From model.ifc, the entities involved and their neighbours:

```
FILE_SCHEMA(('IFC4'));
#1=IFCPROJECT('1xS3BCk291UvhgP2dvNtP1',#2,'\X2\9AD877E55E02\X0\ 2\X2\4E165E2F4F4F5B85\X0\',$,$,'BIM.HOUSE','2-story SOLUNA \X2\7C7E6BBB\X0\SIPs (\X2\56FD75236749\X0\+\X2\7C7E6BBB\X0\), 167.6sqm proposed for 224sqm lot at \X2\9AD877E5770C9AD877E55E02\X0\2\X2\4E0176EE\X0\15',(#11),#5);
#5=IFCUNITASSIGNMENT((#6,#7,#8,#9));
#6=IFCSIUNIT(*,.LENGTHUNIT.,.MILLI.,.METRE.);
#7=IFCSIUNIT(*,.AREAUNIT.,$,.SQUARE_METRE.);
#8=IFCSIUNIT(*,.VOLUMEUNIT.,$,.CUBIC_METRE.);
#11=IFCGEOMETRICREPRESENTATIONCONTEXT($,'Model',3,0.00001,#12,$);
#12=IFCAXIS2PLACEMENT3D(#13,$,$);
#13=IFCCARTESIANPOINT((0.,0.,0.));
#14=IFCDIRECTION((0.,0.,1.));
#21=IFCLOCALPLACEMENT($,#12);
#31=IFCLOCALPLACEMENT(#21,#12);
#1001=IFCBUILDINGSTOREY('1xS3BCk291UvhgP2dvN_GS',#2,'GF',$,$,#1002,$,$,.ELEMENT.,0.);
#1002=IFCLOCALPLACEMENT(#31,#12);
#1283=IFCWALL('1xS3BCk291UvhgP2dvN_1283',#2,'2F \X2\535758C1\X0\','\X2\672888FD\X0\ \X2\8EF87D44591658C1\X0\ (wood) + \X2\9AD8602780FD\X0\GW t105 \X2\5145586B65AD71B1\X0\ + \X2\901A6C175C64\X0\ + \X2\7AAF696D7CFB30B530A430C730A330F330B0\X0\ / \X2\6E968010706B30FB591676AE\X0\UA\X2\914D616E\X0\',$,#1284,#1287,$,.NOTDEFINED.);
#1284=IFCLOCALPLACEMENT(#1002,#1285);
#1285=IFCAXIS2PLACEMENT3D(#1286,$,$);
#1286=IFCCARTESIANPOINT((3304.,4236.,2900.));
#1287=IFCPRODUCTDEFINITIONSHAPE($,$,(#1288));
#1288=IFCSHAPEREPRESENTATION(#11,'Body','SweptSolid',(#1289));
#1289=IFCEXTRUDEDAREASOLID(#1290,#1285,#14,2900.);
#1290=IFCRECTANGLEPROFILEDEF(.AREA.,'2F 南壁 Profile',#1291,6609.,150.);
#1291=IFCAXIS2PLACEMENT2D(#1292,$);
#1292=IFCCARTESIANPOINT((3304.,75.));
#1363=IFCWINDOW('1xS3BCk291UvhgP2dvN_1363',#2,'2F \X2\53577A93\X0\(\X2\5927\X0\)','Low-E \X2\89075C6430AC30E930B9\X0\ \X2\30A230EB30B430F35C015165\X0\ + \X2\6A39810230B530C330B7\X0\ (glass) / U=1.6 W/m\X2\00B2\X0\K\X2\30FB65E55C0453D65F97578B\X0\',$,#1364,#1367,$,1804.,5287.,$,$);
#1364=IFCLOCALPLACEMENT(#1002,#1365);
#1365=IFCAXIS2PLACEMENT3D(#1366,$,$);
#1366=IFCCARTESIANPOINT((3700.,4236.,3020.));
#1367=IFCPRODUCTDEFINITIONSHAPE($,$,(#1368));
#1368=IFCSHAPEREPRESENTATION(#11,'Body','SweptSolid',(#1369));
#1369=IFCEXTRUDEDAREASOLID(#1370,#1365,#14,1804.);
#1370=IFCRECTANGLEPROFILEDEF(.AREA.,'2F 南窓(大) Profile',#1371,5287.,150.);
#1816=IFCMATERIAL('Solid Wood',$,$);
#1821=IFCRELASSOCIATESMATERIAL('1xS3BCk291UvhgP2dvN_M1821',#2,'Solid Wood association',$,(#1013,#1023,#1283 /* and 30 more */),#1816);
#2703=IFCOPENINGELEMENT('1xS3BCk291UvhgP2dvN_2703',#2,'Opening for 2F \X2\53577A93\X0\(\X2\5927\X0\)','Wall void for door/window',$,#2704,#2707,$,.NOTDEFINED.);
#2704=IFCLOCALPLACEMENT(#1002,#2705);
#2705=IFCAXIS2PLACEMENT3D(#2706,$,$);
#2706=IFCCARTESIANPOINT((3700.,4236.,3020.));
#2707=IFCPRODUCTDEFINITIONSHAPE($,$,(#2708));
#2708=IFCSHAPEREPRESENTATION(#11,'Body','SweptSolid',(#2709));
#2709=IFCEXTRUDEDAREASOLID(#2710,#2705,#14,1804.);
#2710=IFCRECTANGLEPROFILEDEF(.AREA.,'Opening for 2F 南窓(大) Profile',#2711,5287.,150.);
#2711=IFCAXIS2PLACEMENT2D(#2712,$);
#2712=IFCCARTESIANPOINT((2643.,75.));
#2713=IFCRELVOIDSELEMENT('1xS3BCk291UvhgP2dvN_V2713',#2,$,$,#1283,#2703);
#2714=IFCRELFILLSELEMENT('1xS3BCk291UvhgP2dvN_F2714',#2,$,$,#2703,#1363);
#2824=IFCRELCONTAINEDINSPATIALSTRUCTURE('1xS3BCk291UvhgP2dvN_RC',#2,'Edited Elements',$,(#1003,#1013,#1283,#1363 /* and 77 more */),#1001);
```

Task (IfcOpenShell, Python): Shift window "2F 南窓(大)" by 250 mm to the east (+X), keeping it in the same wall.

```python
import ifcopenshell
import ifcopenshell.api.geometry
import ifcopenshell.util.placement
import ifcopenshell.util.unit

model = ifcopenshell.open("model.ifc")
unit_scale = ifcopenshell.util.unit.calculate_unit_scale(model)

window = model.by_id(1363)
opening = window.FillsVoids[0].RelatingOpeningElement
wall = opening.VoidsElements[0].RelatingBuildingElement

wall_matrix = ifcopenshell.util.placement.get_local_placement(wall.ObjectPlacement)
shift = wall_matrix[:3, 0] * 0.25 / unit_scale
before = ifcopenshell.util.placement.get_local_placement(window.ObjectPlacement)[:3, 3].copy()

# The window is not placed relative to its opening, so move both.
for product in (opening, window):
    matrix = ifcopenshell.util.placement.get_local_placement(product.ObjectPlacement)
    matrix[:3, 3] += shift
    ifcopenshell.api.geometry.edit_object_placement(model, product=product, matrix=matrix, is_si=False)

after = ifcopenshell.util.placement.get_local_placement(window.ObjectPlacement)[:3, 3]
print("window moved by", (after - before).round(3) + 0.0)

model.write("model_updated.ifc")
```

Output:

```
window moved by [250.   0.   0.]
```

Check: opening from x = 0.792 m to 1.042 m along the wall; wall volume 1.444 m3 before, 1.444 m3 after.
